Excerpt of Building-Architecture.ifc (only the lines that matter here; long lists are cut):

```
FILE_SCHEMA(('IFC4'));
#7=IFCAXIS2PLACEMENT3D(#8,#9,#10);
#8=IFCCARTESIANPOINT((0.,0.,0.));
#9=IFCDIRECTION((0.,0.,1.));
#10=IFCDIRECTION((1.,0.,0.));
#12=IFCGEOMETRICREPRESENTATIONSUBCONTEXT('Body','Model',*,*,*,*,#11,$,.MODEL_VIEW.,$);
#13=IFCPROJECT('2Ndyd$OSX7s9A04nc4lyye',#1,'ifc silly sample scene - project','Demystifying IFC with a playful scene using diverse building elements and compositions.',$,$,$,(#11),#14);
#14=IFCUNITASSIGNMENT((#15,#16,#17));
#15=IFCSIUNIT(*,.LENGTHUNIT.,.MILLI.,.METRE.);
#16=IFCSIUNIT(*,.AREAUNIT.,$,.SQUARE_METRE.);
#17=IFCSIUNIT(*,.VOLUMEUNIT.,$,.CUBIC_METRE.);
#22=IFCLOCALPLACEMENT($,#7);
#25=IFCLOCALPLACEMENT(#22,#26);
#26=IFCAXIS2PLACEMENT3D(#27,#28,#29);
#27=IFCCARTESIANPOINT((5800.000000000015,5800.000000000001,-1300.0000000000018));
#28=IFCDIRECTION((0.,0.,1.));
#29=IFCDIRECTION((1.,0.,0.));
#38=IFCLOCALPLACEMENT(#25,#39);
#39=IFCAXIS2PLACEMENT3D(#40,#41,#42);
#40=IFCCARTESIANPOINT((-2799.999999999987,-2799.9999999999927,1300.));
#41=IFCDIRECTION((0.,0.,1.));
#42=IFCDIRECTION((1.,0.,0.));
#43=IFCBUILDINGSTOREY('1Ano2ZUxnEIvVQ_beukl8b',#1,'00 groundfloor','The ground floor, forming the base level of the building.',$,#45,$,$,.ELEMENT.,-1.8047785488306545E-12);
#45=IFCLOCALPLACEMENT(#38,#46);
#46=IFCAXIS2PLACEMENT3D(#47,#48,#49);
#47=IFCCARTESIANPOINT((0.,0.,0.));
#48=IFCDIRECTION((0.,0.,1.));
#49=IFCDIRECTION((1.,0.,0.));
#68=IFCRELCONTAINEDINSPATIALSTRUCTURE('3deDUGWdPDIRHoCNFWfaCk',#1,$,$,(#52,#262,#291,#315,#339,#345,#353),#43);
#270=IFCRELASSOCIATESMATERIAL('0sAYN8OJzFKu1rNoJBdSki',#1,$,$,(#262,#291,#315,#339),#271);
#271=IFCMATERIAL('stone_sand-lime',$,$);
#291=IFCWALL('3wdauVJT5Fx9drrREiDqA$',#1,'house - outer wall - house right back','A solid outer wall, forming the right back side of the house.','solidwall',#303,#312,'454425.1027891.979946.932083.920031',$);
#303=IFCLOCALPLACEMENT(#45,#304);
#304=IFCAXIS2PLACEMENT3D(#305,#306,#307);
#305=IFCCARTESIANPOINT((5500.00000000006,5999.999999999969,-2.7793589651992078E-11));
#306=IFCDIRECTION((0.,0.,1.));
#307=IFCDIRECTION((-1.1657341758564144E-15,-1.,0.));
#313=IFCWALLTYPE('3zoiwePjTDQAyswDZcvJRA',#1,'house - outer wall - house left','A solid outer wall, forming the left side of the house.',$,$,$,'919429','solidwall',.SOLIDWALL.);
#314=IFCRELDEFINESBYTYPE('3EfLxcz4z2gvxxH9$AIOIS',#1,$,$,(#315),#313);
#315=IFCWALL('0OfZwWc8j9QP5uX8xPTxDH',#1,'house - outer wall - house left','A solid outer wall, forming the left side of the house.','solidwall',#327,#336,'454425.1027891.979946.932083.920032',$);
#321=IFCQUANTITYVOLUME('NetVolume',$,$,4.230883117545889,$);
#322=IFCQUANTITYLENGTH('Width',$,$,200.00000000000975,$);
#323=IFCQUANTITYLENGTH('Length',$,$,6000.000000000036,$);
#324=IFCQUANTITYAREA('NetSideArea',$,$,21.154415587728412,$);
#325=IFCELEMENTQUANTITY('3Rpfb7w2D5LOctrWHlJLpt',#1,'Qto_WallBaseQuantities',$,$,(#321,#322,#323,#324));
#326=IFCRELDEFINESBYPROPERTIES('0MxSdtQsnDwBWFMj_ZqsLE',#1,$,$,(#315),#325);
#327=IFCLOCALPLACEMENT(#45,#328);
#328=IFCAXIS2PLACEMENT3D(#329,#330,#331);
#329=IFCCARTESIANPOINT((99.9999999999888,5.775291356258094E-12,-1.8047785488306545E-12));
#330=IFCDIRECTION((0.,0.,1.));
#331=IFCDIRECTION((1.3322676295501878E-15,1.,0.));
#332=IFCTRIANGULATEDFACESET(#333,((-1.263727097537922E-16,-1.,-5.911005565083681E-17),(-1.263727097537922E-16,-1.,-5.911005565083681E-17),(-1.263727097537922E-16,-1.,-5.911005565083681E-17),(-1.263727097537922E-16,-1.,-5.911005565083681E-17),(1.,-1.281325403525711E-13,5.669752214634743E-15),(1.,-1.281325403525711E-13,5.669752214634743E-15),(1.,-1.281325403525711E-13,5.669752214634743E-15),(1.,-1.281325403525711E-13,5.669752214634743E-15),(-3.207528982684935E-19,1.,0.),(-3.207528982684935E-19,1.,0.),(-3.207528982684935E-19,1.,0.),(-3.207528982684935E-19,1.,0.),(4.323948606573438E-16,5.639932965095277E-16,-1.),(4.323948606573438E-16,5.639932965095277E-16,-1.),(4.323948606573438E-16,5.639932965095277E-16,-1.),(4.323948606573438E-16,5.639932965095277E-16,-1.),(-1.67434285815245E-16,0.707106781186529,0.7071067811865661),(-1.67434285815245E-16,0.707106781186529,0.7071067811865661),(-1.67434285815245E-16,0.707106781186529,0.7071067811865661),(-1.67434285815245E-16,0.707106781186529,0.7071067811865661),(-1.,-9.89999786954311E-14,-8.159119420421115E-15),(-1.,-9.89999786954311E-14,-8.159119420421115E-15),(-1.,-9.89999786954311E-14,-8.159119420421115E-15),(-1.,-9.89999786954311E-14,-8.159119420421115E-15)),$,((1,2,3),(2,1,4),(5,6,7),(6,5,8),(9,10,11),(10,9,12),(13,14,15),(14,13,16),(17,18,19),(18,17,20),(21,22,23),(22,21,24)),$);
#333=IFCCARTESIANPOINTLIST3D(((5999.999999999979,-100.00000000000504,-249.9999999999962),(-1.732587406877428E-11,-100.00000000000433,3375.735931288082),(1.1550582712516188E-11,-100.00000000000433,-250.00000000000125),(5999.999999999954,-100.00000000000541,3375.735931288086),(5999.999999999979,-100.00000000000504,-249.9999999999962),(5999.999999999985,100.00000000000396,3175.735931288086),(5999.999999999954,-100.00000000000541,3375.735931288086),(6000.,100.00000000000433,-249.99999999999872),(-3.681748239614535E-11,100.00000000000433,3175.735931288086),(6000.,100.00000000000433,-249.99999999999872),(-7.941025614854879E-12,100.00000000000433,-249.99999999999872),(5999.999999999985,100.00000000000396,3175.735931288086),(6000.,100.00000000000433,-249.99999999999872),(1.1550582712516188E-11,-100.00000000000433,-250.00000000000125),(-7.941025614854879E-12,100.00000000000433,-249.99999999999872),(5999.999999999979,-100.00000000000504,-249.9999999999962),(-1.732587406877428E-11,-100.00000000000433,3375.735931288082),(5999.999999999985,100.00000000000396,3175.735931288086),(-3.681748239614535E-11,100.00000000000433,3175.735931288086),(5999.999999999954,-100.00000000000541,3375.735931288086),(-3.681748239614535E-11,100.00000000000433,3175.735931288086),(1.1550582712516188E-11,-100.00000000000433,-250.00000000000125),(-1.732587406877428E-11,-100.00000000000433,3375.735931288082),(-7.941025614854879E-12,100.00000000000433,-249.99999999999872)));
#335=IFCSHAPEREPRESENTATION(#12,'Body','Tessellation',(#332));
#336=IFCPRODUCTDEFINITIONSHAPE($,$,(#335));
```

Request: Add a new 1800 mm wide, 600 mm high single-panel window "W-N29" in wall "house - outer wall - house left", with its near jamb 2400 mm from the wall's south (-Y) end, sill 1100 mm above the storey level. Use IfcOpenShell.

```python
import numpy as np
import ifcopenshell
import ifcopenshell.api.feature
import ifcopenshell.api.geometry
import ifcopenshell.api.pset
import ifcopenshell.api.root
import ifcopenshell.api.spatial
import ifcopenshell.geom
import ifcopenshell.util.element
import ifcopenshell.util.placement
import ifcopenshell.util.representation
import ifcopenshell.util.shape
import ifcopenshell.util.unit

model = ifcopenshell.open("Building-Architecture.ifc")
unit_scale = ifcopenshell.util.unit.calculate_unit_scale(model)
area_scale = ifcopenshell.util.unit.calculate_unit_scale(model, "AREAUNIT")
volume_scale = ifcopenshell.util.unit.calculate_unit_scale(model, "VOLUMEUNIT")
settings = ifcopenshell.geom.settings()


def volume(element):
    """Net volume in cubic metres, openings subtracted."""
    shape = ifcopenshell.geom.create_shape(settings, element)
    return ifcopenshell.util.shape.get_volume(shape.geometry)


wall = model.by_guid("0OfZwWc8j9QP5uX8xPTxDH")
storey = ifcopenshell.util.element.get_container(wall, ifc_class="IfcBuildingStorey")
context = ifcopenshell.util.representation.get_context(model, "Model", "Body", "MODEL_VIEW")
before = volume(wall)

width, height, from_end, sill = 1.8, 0.6, 2.4, 1.1  # metres

# The wall runs along its own X axis, and the end named is its -X end.
wall_shape = ifcopenshell.geom.create_shape(settings, wall)
x, y, z = ifcopenshell.util.shape.get_vertices(wall_shape.geometry).T
start = x.min() + from_end
face, thickness = float(y.min()), float(y.max() - y.min())
wall_matrix = ifcopenshell.util.placement.get_local_placement(wall.ObjectPlacement)
level = ifcopenshell.util.placement.get_local_placement(storey.ObjectPlacement)[2, 3]


def in_wall(x, y):
    """Placement at x, y metres in the wall's axes, at sill height."""
    matrix = wall_matrix.copy()
    matrix[:, 3] = wall_matrix @ np.array([x / unit_scale, y / unit_scale, 0.0, 1.0])
    matrix[2, 3] = level + sill / unit_scale
    return matrix


# Opening: a box that overshoots both wall faces by 50 mm.
opening = ifcopenshell.api.root.create_entity(model, ifc_class="IfcOpeningElement", predefined_type="OPENING")
box = ifcopenshell.api.geometry.add_wall_representation(
    model, context=context, length=width, height=height, thickness=thickness + 0.1
)
ifcopenshell.api.geometry.assign_representation(model, product=opening, representation=box)
ifcopenshell.api.geometry.edit_object_placement(model, product=opening, matrix=in_wall(start, face - 0.05), is_si=False)
ifcopenshell.api.feature.add_feature(model, feature=opening, element=wall)

window = ifcopenshell.api.root.create_entity(model, ifc_class="IfcWindow", name="W-N29", predefined_type="WINDOW")
window.OverallWidth, window.OverallHeight = width / unit_scale, height / unit_scale
window.PartitioningType = "SINGLE_PANEL"
body = ifcopenshell.api.geometry.add_window_representation(
    model,
    context=context,
    overall_width=window.OverallWidth,
    overall_height=window.OverallHeight,
    partition_type="SINGLE_PANEL",
)
ifcopenshell.api.geometry.assign_representation(model, product=window, representation=body)
ifcopenshell.api.spatial.assign_container(model, products=[window], relating_structure=storey)
ifcopenshell.api.feature.add_filling(model, opening=opening, element=window)

# Centre the window in the wall's thickness.
ifcopenshell.api.geometry.edit_object_placement(model, product=window, matrix=in_wall(start, face), is_si=False)
window_shape = ifcopenshell.geom.create_shape(settings, window)
depth = ifcopenshell.util.shape.get_vertices(window_shape.geometry)[:, 1]
offset = face + thickness / 2 - (depth.min() + depth.max()) / 2
ifcopenshell.api.geometry.edit_object_placement(model, product=window, matrix=in_wall(start, offset), is_si=False)

after = volume(wall)

# Update the wall's stored quantities.
qto = model.by_id(ifcopenshell.util.element.get_pset(wall, "Qto_WallBaseQuantities", should_inherit=False)["id"])
ifcopenshell.api.pset.edit_qto(model, qto=qto, properties={
    "NetVolume": after / volume_scale,
    "NetSideArea": after / thickness / area_scale,
})

print(f"wall volume {before:.3f} -> {after:.3f} m3")

model.write("Building-Architecture_rev.ifc")
```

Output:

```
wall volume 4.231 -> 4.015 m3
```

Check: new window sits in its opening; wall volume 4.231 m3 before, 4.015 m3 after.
